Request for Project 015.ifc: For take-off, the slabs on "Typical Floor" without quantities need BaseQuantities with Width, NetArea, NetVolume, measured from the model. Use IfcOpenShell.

First a look at what the model holds.

```python
import ifcopenshell
import ifcopenshell.util.element
import ifcopenshell.util.unit

model = ifcopenshell.open("Project 015.ifc")
print(model.schema)
for unit_type in ("LENGTHUNIT", "AREAUNIT", "VOLUMEUNIT"):
    print(unit_type, ifcopenshell.util.unit.calculate_unit_scale(model, unit_type))
storey = next(s for s in model.by_type("IfcBuildingStorey") if s.Name == "Typical Floor")
slabs = [e for e in ifcopenshell.util.element.get_decomposition(storey) if e.is_a("IfcSlab")]
for e in sorted(slabs, key=lambda e: e.id()):
    print(e.id(), e.is_a(), e.Name, list(ifcopenshell.util.element.get_psets(e, qtos_only=True)), sep=" | ")
```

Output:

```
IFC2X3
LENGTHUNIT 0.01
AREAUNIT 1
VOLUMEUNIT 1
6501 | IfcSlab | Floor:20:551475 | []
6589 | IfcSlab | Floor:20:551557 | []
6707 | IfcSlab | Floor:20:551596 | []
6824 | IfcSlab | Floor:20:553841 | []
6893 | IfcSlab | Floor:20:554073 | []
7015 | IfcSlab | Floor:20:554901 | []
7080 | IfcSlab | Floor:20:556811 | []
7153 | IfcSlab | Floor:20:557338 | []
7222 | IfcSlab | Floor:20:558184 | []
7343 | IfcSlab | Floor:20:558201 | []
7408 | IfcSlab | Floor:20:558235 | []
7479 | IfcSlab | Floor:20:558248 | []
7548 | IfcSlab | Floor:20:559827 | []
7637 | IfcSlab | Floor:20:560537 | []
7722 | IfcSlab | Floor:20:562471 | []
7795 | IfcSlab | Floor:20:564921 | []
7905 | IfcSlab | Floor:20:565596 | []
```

```python
import ifcopenshell
import ifcopenshell.api.pset
import ifcopenshell.geom
import ifcopenshell.util.element
import ifcopenshell.util.shape
import ifcopenshell.util.unit

model = ifcopenshell.open("Project 015.ifc")
unit_scale = ifcopenshell.util.unit.calculate_unit_scale(model)
area_scale = ifcopenshell.util.unit.calculate_unit_scale(model, "AREAUNIT")
volume_scale = ifcopenshell.util.unit.calculate_unit_scale(model, "VOLUMEUNIT")
settings = ifcopenshell.geom.settings()

storey = next(s for s in model.by_type("IfcBuildingStorey") if s.Name == "Typical Floor")
slabs = [e for e in ifcopenshell.util.element.get_decomposition(storey) if e.is_a("IfcSlab")]

for e in sorted(slabs, key=lambda e: e.id()):
    if ifcopenshell.util.element.get_psets(e, qtos_only=True, should_inherit=False):
        continue
    # Geometry comes back in metres, in the element's own axes.
    shape = ifcopenshell.geom.create_shape(settings, e)
    values = {
        "Width": ifcopenshell.util.shape.get_z(shape.geometry) / unit_scale,
        "NetArea": ifcopenshell.util.shape.get_footprint_area(shape.geometry) / area_scale,
        "NetVolume": ifcopenshell.util.shape.get_volume(shape.geometry) / volume_scale,
    }
    qto = ifcopenshell.api.pset.add_qto(model, product=e, name="BaseQuantities")
    ifcopenshell.api.pset.edit_qto(model, qto=qto, properties=values)
    print(e.id(), {k: round(v, 3) for k, v in values.items()})

model.write("Project 015-out.ifc")
```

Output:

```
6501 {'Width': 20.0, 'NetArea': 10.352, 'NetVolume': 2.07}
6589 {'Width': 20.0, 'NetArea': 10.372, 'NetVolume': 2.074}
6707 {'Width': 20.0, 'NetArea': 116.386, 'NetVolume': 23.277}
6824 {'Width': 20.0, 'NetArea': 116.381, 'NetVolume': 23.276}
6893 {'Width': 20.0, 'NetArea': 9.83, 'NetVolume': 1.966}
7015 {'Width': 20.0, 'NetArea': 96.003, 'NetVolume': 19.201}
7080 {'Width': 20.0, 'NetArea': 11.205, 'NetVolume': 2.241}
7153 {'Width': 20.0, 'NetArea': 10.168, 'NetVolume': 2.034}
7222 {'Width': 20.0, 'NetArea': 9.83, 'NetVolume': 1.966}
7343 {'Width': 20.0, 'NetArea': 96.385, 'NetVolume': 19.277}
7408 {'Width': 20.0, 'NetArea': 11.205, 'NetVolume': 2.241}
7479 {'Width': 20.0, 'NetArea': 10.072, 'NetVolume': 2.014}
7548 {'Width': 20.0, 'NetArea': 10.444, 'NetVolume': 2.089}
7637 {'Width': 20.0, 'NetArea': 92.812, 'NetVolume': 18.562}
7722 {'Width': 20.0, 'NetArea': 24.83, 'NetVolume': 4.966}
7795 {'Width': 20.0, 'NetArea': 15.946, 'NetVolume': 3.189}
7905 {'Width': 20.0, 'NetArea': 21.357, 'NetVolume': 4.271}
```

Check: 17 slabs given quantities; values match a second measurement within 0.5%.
